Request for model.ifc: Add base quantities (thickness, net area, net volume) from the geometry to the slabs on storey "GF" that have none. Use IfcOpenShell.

First a look at what the model holds.

```python
import ifcopenshell
import ifcopenshell.util.element
import ifcopenshell.util.unit

model = ifcopenshell.open("model.ifc")
print(model.schema)
for unit_type in ("LENGTHUNIT", "AREAUNIT", "VOLUMEUNIT"):
    print(unit_type, ifcopenshell.util.unit.calculate_unit_scale(model, unit_type))
storey = next(s for s in model.by_type("IfcBuildingStorey") if s.Name == "GF")
slabs = [e for e in ifcopenshell.util.element.get_decomposition(storey) if e.is_a("IfcSlab")]
for e in sorted(slabs, key=lambda e: e.id()):
    print(e.id(), e.is_a(), e.Name, list(ifcopenshell.util.element.get_psets(e, qtos_only=True)), sep=" | ")
```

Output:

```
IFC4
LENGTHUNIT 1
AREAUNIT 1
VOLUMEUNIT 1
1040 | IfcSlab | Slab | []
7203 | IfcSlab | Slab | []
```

```python
import ifcopenshell
import ifcopenshell.api.pset
import ifcopenshell.geom
import ifcopenshell.util.element
import ifcopenshell.util.shape
import ifcopenshell.util.unit

model = ifcopenshell.open("model.ifc")
unit_scale = ifcopenshell.util.unit.calculate_unit_scale(model)
area_scale = ifcopenshell.util.unit.calculate_unit_scale(model, "AREAUNIT")
volume_scale = ifcopenshell.util.unit.calculate_unit_scale(model, "VOLUMEUNIT")
settings = ifcopenshell.geom.settings()

storey = next(s for s in model.by_type("IfcBuildingStorey") if s.Name == "GF")
slabs = [e for e in ifcopenshell.util.element.get_decomposition(storey) if e.is_a("IfcSlab")]

for e in sorted(slabs, key=lambda e: e.id()):
    if ifcopenshell.util.element.get_psets(e, qtos_only=True, should_inherit=False):
        continue
    # Geometry comes back in metres, in the element's own axes.
    shape = ifcopenshell.geom.create_shape(settings, e)
    values = {
        "Width": ifcopenshell.util.shape.get_z(shape.geometry) / unit_scale,
        "NetArea": ifcopenshell.util.shape.get_footprint_area(shape.geometry) / area_scale,
        "NetVolume": ifcopenshell.util.shape.get_volume(shape.geometry) / volume_scale,
    }
    qto = ifcopenshell.api.pset.add_qto(model, product=e, name="Qto_SlabBaseQuantities")
    ifcopenshell.api.pset.edit_qto(model, qto=qto, properties=values)
    print(e.id(), {k: round(v, 3) for k, v in values.items()})

model.write("model_edited.ifc")
```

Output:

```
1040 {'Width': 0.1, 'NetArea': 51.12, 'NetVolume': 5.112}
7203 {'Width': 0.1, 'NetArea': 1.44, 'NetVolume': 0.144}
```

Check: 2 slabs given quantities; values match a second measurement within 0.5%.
